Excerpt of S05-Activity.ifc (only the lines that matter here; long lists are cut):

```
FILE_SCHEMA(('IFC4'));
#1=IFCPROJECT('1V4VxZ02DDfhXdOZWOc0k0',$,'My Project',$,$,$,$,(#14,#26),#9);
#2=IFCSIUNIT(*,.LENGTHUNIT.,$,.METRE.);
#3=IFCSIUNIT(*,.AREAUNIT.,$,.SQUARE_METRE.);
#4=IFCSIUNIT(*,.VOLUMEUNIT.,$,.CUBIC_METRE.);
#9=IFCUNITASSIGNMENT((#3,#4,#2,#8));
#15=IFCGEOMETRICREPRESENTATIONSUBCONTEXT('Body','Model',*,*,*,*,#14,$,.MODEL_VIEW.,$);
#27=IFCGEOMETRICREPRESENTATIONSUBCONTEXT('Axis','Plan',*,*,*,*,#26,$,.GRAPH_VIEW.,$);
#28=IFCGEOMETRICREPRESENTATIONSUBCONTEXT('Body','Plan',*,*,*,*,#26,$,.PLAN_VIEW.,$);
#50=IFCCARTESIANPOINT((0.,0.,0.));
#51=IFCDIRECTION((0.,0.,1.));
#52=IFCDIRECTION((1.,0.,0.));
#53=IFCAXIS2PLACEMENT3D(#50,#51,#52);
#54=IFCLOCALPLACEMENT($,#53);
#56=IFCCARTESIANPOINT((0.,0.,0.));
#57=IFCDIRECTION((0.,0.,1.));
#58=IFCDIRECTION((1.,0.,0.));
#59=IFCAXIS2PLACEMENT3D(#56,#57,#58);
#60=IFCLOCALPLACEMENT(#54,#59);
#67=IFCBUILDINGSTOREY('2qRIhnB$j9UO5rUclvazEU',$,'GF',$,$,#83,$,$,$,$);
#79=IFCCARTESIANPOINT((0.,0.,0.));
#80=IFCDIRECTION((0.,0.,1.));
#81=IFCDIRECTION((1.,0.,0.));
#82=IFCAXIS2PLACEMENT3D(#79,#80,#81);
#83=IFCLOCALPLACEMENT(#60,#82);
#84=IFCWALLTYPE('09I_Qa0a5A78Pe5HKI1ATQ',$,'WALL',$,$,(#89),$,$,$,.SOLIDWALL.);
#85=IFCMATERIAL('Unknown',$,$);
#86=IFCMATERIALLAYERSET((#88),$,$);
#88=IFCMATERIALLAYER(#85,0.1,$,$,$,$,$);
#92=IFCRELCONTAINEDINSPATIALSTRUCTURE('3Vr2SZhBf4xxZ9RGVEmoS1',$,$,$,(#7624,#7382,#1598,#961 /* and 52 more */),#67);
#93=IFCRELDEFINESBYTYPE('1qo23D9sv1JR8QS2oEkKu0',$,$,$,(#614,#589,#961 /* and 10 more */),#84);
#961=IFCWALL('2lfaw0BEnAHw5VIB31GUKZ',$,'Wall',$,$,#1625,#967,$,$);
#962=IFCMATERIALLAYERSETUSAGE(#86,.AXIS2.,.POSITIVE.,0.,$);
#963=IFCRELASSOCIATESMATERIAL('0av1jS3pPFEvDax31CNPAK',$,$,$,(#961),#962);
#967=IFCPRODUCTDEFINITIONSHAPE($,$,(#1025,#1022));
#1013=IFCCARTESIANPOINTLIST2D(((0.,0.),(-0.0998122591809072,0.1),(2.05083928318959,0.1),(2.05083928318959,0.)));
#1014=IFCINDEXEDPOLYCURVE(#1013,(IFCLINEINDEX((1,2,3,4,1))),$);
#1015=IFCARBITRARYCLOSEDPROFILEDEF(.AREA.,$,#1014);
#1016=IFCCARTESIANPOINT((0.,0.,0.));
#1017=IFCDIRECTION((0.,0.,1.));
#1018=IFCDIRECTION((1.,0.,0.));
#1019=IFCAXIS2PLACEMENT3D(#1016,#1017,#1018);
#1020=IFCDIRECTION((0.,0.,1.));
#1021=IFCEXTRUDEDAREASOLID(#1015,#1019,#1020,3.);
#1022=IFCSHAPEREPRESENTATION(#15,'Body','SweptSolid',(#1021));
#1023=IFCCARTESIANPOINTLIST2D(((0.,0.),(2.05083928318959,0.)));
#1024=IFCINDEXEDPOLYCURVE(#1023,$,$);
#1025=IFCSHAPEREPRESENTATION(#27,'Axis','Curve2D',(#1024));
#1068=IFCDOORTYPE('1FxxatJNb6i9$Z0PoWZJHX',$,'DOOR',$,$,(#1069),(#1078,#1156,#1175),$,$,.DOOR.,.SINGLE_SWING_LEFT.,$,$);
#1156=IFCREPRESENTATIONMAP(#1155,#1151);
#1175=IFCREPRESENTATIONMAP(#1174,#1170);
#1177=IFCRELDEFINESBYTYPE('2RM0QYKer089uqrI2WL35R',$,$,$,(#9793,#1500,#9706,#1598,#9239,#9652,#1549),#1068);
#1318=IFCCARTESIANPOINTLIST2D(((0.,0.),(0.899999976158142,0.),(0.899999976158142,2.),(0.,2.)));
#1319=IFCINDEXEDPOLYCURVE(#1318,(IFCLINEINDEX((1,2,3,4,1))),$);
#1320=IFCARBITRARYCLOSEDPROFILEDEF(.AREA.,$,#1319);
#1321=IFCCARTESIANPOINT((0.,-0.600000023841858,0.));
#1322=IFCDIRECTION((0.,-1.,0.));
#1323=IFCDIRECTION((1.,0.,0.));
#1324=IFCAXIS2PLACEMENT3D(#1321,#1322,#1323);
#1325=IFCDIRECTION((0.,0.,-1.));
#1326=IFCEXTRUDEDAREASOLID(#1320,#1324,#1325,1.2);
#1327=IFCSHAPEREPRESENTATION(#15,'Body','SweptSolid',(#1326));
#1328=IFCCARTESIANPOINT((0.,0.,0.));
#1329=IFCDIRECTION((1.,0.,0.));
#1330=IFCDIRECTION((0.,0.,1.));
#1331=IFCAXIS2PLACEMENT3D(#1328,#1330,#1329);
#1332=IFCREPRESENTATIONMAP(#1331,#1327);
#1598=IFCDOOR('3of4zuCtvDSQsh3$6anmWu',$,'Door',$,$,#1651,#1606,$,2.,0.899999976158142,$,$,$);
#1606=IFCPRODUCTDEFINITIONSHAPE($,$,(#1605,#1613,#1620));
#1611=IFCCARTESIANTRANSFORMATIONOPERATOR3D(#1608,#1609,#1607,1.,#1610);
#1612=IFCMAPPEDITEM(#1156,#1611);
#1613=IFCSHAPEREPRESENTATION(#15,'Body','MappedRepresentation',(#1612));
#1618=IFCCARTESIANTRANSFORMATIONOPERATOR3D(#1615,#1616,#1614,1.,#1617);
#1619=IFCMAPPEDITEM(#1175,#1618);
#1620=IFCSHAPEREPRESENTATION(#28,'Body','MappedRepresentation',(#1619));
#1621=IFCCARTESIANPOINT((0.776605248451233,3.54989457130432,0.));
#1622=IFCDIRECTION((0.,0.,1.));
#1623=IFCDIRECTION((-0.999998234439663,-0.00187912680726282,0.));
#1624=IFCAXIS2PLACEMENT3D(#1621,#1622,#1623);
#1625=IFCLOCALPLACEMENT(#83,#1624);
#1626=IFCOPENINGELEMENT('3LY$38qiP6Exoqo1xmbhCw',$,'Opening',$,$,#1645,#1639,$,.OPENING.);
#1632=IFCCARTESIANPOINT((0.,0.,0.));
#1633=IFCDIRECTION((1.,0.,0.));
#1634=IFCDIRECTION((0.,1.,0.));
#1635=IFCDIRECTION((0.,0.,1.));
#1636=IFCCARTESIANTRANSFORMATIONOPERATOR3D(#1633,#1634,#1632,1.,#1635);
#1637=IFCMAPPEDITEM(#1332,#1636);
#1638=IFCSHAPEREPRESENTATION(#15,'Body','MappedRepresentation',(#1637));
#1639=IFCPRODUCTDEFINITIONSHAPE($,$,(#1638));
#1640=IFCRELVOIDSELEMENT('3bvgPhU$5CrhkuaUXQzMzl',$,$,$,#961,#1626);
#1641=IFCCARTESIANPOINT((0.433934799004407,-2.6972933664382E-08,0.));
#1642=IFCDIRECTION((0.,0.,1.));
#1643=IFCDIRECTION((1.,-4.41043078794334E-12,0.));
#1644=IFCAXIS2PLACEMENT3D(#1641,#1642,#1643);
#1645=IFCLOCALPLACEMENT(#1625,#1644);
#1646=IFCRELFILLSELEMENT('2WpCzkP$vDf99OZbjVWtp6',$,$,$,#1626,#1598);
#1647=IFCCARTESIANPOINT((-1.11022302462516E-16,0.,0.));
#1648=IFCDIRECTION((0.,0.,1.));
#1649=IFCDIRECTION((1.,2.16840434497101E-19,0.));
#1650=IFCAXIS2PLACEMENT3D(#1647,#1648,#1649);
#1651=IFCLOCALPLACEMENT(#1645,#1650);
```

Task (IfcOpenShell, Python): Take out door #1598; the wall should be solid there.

```python
import ifcopenshell
import ifcopenshell.api.feature
import ifcopenshell.api.root
import ifcopenshell.geom
import ifcopenshell.util.shape

model = ifcopenshell.open("S05-Activity.ifc")
settings = ifcopenshell.geom.settings()


def volume(element):
    """Net volume in cubic metres, openings subtracted."""
    shape = ifcopenshell.geom.create_shape(settings, element)
    return ifcopenshell.util.shape.get_volume(shape.geometry)


door = model.by_guid("3of4zuCtvDSQsh3$6anmWu")
opening = door.FillsVoids[0].RelatingOpeningElement
wall = opening.VoidsElements[0].RelatingBuildingElement
before = volume(wall)

ifcopenshell.api.root.remove_product(model, product=door)
ifcopenshell.api.feature.remove_feature(model, feature=opening)

after = volume(wall)

print(f"wall volume {before:.3f} -> {after:.3f} m3")

model.write("S05-Activity_v2.ifc")
```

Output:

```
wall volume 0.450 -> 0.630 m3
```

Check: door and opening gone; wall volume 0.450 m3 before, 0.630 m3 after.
